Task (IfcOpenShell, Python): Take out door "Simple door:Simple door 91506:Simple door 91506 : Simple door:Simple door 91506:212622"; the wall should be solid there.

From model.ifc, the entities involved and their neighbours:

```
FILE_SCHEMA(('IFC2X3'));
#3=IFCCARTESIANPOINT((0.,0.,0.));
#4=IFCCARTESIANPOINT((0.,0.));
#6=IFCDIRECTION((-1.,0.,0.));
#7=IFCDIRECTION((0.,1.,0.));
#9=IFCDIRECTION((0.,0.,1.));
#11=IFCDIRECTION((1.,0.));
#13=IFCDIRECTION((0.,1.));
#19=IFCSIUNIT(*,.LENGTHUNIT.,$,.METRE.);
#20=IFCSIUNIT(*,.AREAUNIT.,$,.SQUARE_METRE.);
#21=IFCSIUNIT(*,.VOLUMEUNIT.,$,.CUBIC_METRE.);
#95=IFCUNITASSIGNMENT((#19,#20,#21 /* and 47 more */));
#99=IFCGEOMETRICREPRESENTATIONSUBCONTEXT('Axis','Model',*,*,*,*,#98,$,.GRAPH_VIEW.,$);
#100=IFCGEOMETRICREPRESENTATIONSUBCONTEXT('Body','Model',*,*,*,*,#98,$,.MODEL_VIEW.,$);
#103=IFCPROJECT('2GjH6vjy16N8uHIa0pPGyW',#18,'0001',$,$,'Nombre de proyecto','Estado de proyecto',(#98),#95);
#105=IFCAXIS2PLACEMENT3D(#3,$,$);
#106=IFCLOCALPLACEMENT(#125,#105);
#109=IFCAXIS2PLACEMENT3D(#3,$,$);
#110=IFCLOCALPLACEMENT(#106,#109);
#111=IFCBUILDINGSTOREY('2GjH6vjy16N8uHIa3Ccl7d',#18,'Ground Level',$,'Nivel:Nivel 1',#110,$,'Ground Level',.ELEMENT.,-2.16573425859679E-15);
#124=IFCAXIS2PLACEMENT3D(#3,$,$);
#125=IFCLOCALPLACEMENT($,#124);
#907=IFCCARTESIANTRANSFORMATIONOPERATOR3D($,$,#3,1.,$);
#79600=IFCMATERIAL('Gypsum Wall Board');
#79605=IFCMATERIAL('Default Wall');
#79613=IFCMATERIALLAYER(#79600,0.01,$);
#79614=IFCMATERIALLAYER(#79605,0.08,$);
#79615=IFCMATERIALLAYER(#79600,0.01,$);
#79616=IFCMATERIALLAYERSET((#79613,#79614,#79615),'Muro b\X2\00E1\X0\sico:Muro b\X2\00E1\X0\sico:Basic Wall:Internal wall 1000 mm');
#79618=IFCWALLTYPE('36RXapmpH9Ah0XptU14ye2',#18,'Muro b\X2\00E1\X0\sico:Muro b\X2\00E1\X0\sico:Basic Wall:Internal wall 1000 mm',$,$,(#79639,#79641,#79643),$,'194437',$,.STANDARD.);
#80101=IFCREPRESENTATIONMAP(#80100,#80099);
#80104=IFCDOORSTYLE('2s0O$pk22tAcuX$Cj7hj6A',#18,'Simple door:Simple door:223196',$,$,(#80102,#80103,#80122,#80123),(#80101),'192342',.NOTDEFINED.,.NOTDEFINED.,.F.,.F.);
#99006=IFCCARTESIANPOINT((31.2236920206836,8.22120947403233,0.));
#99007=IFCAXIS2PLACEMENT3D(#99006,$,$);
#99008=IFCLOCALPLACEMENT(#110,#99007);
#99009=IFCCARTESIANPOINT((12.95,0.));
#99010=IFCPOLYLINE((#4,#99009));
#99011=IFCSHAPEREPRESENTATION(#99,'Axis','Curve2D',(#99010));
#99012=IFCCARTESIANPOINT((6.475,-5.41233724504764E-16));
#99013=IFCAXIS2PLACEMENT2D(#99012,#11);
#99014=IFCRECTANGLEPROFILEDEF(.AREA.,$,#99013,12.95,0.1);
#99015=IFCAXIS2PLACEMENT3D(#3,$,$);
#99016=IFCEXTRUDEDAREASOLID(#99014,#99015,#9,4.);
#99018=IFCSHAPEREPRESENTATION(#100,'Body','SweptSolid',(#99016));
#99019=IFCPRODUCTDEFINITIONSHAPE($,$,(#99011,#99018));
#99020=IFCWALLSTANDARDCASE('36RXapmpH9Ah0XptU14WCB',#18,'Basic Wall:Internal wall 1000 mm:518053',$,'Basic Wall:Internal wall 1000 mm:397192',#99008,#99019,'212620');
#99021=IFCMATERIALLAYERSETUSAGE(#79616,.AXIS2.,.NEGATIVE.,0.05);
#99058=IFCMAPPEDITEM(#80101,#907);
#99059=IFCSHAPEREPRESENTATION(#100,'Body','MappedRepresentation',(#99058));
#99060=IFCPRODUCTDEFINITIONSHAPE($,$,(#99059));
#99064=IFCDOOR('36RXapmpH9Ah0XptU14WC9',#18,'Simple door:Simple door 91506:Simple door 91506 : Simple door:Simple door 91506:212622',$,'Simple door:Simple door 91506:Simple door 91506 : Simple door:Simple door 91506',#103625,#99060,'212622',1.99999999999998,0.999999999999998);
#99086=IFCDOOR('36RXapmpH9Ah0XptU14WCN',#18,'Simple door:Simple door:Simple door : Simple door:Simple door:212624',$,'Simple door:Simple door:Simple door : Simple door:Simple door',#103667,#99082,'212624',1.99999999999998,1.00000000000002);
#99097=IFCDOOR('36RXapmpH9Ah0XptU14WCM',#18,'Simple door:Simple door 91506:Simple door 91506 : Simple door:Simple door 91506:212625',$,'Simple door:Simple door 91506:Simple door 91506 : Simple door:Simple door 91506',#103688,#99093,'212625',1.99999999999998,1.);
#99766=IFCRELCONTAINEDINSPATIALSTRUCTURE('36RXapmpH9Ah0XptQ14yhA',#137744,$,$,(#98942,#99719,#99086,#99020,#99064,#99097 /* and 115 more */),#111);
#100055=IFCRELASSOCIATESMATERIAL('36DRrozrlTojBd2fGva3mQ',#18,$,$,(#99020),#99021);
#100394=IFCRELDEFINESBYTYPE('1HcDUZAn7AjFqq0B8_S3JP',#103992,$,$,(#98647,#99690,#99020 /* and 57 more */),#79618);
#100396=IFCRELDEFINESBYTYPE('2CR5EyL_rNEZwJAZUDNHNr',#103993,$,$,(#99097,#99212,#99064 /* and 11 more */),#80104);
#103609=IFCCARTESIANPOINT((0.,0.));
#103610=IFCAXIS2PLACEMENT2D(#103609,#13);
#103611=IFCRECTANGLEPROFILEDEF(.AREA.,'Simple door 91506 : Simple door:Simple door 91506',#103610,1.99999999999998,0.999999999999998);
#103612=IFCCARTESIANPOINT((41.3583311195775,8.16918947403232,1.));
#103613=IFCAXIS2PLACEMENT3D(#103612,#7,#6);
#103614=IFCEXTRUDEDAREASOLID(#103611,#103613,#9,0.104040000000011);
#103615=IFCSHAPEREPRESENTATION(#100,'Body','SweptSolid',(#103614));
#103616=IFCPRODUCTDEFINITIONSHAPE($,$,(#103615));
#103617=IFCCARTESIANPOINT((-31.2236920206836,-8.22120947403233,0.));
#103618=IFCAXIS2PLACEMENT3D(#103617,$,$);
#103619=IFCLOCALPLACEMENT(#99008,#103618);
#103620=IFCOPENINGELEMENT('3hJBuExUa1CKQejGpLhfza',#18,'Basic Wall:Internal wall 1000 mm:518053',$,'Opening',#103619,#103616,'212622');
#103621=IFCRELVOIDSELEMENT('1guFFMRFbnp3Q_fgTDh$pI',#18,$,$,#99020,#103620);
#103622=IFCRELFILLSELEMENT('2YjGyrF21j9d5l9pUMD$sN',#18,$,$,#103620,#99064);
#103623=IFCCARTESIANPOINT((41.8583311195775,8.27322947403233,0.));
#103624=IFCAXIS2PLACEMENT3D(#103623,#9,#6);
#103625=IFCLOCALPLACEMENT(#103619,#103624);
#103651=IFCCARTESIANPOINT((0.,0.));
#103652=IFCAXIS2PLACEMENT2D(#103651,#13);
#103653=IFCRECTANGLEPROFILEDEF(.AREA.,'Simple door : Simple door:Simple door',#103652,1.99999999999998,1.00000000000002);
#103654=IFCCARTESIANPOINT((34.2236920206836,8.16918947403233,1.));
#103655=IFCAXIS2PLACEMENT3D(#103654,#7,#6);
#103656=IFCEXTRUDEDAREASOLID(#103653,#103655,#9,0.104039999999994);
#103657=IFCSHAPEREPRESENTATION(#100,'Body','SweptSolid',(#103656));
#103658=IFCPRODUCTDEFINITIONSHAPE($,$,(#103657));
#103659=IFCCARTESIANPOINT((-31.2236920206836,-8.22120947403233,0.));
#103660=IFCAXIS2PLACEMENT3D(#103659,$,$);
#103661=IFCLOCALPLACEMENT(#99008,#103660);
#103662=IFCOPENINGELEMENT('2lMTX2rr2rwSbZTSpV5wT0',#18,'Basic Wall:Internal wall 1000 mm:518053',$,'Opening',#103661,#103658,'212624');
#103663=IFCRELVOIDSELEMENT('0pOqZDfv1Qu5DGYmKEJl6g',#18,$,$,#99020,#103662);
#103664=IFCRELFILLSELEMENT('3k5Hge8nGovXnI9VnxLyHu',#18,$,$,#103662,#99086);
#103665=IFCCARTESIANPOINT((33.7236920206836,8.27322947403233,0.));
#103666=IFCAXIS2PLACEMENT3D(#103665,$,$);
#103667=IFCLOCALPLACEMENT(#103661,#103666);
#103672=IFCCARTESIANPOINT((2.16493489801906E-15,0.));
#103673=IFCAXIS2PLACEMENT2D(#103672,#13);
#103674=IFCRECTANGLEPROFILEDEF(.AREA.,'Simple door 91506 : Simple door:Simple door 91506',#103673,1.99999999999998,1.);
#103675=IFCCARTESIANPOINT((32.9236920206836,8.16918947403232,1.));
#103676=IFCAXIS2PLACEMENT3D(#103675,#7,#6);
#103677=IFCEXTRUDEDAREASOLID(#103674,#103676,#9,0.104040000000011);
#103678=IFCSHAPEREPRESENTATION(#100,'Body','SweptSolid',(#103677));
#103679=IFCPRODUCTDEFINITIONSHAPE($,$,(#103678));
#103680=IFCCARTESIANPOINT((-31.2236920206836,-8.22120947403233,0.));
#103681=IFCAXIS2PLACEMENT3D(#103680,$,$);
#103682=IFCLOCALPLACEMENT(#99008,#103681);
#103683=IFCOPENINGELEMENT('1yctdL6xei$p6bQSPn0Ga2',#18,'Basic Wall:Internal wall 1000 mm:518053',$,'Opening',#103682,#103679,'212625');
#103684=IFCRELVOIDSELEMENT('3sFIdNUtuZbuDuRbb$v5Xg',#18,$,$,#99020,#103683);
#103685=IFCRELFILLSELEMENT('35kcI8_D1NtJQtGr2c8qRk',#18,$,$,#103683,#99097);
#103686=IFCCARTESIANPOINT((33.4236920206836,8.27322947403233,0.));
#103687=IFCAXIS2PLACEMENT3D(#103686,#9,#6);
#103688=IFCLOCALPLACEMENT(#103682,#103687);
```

```python
import ifcopenshell
import ifcopenshell.api.feature
import ifcopenshell.api.root
import ifcopenshell.geom
import ifcopenshell.util.shape

model = ifcopenshell.open("model.ifc")
settings = ifcopenshell.geom.settings()


def volume(element):
    """Net volume in cubic metres, openings subtracted."""
    shape = ifcopenshell.geom.create_shape(settings, element)
    return ifcopenshell.util.shape.get_volume(shape.geometry)


door = model.by_guid("36RXapmpH9Ah0XptU14WC9")
opening = door.FillsVoids[0].RelatingOpeningElement
wall = opening.VoidsElements[0].RelatingBuildingElement
before = volume(wall)

ifcopenshell.api.root.remove_product(model, product=door)
ifcopenshell.api.feature.remove_feature(model, feature=opening)

after = volume(wall)

print(f"wall volume {before:.3f} -> {after:.3f} m3")

model.write("model-out.ifc")
```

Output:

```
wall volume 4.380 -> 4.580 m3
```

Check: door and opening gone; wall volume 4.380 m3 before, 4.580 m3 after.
